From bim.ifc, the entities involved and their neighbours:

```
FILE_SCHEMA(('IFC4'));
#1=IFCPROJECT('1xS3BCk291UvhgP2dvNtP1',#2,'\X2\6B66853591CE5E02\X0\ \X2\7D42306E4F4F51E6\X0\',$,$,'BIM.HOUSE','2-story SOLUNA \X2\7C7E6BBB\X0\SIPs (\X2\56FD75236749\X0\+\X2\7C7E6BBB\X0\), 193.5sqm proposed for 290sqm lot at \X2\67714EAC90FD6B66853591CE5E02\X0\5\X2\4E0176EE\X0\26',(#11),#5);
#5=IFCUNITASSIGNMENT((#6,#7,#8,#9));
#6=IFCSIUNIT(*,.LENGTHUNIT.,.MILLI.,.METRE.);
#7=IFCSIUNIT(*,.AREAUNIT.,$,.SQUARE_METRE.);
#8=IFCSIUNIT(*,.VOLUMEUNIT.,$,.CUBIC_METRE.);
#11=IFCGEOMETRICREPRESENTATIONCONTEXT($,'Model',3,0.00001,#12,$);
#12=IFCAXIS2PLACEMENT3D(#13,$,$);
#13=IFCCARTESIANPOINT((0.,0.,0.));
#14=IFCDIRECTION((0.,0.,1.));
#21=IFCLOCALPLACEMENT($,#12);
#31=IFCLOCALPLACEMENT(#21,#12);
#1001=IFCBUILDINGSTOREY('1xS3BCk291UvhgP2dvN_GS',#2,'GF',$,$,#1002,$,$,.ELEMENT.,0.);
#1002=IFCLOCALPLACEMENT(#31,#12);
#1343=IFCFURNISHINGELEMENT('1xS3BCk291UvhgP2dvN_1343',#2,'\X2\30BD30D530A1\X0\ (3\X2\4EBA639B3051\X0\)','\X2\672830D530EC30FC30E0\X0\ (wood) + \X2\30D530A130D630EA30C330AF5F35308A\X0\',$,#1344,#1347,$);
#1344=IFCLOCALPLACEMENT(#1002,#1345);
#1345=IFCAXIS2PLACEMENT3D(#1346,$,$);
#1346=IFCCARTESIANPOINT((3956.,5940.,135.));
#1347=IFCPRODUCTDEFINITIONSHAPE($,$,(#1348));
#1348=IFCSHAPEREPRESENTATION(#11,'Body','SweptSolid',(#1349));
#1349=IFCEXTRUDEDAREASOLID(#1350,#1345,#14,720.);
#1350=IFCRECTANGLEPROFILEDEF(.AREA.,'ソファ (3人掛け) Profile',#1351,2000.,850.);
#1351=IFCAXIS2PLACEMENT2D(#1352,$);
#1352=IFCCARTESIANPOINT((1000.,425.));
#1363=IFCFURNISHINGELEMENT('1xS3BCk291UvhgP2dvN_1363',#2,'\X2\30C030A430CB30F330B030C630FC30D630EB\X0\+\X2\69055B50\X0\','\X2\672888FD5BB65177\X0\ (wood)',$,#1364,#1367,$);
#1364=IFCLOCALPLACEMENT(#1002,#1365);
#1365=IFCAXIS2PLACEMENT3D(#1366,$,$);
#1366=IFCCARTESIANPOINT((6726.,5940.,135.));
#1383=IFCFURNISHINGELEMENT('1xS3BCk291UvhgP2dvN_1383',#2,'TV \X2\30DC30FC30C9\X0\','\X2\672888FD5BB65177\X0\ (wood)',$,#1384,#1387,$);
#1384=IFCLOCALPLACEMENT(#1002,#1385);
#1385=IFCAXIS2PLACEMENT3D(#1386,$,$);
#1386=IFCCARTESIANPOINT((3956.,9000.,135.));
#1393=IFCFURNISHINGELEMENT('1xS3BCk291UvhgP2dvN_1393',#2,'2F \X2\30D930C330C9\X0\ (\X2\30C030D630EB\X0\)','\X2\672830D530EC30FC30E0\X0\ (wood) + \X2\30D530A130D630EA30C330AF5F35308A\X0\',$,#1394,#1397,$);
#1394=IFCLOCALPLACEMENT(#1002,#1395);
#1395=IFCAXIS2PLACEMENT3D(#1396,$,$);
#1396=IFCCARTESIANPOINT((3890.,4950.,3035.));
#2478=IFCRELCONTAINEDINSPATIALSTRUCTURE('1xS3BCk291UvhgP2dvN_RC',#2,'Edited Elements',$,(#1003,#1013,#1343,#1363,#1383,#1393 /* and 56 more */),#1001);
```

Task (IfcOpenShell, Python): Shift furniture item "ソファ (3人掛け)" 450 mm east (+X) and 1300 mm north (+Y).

```python
import ifcopenshell
import ifcopenshell.api.geometry
import ifcopenshell.util.placement
import ifcopenshell.util.unit

model = ifcopenshell.open("bim.ifc")
unit_scale = ifcopenshell.util.unit.calculate_unit_scale(model)

item = model.by_guid("1xS3BCk291UvhgP2dvN_1343")
matrix = ifcopenshell.util.placement.get_local_placement(item.ObjectPlacement)
matrix[0, 3] += 0.45 / unit_scale
matrix[1, 3] += 1.3 / unit_scale
ifcopenshell.api.geometry.edit_object_placement(model, product=item, matrix=matrix, is_si=False)

print(ifcopenshell.util.placement.get_local_placement(item.ObjectPlacement).round(3) + 0.0)

model.write("bim_edited.ifc")
```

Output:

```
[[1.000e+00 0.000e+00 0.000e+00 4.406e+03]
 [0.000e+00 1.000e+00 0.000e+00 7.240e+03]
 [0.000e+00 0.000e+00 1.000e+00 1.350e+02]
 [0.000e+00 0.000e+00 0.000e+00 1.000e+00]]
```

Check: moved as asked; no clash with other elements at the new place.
